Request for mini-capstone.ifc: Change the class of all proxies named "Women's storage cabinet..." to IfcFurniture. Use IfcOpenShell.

First a look at what the model holds.

```python
import re

import ifcopenshell

model = ifcopenshell.open("mini-capstone.ifc")
print(model.schema)
seen = {}
for e in model.by_type("IfcBuildingElementProxy"):
    name = re.sub(r":\d+(:\d+)?$", "", e.Name or "")  # drop the element id that some exporters append
    seen[name] = seen.get(name, 0) + 1
for name, count in sorted(seen.items()):
    print(count, "x", name)
```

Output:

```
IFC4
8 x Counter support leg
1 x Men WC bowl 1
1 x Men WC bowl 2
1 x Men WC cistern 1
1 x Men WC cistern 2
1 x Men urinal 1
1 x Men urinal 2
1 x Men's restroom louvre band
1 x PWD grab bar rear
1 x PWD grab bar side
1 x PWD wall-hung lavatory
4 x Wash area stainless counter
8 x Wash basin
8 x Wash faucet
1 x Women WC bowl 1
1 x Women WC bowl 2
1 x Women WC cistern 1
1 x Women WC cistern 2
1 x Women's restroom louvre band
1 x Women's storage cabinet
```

```python
import ifcopenshell
import ifcopenshell.api.root

model = ifcopenshell.open("mini-capstone.ifc")

proxies = [e.id() for e in model.by_type("IfcBuildingElementProxy") if (e.Name or "").startswith("Women's storage cabinet")]
for step_id in proxies:
    proxy = model.by_id(step_id)
    ifcopenshell.api.root.reassign_class(model, product=proxy, ifc_class="IfcFurniture")

print(sum(model.by_id(i).is_a("IfcFurniture") for i in proxies), "reclassified")

model.write("mini-capstone-out.ifc")
```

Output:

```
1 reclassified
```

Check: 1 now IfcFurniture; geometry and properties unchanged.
